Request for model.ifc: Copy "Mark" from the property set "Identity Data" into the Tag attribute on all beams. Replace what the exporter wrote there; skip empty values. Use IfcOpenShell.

First a look at what the model holds.

```python
import ifcopenshell
import ifcopenshell.util.element

model = ifcopenshell.open("model.ifc")
print(model.schema)
beams = model.by_type("IfcBeam")
print(len(beams), "beams")
for e in beams[:8]:
    source = ifcopenshell.util.element.get_pset(e, "Identity Data", "Mark")
    target = e.Tag
    print(e.id(), repr(source), repr(target), sep=" | ")
```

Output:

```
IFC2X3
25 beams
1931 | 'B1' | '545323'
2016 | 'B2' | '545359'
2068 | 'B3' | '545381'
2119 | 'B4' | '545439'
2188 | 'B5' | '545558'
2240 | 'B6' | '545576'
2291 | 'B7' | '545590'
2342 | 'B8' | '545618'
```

```python
import ifcopenshell
import ifcopenshell.util.element

model = ifcopenshell.open("model.ifc")

count = 0
for e in model.by_type("IfcBeam"):
    value = ifcopenshell.util.element.get_pset(e, "Identity Data", "Mark")
    current = e.Tag
    if not value or not value.strip() or current == value:
        continue
    e.Tag = value
    count += 1

print(count, "beams updated")

model.write("model_edited.ifc")
```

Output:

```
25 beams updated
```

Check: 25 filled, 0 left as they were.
